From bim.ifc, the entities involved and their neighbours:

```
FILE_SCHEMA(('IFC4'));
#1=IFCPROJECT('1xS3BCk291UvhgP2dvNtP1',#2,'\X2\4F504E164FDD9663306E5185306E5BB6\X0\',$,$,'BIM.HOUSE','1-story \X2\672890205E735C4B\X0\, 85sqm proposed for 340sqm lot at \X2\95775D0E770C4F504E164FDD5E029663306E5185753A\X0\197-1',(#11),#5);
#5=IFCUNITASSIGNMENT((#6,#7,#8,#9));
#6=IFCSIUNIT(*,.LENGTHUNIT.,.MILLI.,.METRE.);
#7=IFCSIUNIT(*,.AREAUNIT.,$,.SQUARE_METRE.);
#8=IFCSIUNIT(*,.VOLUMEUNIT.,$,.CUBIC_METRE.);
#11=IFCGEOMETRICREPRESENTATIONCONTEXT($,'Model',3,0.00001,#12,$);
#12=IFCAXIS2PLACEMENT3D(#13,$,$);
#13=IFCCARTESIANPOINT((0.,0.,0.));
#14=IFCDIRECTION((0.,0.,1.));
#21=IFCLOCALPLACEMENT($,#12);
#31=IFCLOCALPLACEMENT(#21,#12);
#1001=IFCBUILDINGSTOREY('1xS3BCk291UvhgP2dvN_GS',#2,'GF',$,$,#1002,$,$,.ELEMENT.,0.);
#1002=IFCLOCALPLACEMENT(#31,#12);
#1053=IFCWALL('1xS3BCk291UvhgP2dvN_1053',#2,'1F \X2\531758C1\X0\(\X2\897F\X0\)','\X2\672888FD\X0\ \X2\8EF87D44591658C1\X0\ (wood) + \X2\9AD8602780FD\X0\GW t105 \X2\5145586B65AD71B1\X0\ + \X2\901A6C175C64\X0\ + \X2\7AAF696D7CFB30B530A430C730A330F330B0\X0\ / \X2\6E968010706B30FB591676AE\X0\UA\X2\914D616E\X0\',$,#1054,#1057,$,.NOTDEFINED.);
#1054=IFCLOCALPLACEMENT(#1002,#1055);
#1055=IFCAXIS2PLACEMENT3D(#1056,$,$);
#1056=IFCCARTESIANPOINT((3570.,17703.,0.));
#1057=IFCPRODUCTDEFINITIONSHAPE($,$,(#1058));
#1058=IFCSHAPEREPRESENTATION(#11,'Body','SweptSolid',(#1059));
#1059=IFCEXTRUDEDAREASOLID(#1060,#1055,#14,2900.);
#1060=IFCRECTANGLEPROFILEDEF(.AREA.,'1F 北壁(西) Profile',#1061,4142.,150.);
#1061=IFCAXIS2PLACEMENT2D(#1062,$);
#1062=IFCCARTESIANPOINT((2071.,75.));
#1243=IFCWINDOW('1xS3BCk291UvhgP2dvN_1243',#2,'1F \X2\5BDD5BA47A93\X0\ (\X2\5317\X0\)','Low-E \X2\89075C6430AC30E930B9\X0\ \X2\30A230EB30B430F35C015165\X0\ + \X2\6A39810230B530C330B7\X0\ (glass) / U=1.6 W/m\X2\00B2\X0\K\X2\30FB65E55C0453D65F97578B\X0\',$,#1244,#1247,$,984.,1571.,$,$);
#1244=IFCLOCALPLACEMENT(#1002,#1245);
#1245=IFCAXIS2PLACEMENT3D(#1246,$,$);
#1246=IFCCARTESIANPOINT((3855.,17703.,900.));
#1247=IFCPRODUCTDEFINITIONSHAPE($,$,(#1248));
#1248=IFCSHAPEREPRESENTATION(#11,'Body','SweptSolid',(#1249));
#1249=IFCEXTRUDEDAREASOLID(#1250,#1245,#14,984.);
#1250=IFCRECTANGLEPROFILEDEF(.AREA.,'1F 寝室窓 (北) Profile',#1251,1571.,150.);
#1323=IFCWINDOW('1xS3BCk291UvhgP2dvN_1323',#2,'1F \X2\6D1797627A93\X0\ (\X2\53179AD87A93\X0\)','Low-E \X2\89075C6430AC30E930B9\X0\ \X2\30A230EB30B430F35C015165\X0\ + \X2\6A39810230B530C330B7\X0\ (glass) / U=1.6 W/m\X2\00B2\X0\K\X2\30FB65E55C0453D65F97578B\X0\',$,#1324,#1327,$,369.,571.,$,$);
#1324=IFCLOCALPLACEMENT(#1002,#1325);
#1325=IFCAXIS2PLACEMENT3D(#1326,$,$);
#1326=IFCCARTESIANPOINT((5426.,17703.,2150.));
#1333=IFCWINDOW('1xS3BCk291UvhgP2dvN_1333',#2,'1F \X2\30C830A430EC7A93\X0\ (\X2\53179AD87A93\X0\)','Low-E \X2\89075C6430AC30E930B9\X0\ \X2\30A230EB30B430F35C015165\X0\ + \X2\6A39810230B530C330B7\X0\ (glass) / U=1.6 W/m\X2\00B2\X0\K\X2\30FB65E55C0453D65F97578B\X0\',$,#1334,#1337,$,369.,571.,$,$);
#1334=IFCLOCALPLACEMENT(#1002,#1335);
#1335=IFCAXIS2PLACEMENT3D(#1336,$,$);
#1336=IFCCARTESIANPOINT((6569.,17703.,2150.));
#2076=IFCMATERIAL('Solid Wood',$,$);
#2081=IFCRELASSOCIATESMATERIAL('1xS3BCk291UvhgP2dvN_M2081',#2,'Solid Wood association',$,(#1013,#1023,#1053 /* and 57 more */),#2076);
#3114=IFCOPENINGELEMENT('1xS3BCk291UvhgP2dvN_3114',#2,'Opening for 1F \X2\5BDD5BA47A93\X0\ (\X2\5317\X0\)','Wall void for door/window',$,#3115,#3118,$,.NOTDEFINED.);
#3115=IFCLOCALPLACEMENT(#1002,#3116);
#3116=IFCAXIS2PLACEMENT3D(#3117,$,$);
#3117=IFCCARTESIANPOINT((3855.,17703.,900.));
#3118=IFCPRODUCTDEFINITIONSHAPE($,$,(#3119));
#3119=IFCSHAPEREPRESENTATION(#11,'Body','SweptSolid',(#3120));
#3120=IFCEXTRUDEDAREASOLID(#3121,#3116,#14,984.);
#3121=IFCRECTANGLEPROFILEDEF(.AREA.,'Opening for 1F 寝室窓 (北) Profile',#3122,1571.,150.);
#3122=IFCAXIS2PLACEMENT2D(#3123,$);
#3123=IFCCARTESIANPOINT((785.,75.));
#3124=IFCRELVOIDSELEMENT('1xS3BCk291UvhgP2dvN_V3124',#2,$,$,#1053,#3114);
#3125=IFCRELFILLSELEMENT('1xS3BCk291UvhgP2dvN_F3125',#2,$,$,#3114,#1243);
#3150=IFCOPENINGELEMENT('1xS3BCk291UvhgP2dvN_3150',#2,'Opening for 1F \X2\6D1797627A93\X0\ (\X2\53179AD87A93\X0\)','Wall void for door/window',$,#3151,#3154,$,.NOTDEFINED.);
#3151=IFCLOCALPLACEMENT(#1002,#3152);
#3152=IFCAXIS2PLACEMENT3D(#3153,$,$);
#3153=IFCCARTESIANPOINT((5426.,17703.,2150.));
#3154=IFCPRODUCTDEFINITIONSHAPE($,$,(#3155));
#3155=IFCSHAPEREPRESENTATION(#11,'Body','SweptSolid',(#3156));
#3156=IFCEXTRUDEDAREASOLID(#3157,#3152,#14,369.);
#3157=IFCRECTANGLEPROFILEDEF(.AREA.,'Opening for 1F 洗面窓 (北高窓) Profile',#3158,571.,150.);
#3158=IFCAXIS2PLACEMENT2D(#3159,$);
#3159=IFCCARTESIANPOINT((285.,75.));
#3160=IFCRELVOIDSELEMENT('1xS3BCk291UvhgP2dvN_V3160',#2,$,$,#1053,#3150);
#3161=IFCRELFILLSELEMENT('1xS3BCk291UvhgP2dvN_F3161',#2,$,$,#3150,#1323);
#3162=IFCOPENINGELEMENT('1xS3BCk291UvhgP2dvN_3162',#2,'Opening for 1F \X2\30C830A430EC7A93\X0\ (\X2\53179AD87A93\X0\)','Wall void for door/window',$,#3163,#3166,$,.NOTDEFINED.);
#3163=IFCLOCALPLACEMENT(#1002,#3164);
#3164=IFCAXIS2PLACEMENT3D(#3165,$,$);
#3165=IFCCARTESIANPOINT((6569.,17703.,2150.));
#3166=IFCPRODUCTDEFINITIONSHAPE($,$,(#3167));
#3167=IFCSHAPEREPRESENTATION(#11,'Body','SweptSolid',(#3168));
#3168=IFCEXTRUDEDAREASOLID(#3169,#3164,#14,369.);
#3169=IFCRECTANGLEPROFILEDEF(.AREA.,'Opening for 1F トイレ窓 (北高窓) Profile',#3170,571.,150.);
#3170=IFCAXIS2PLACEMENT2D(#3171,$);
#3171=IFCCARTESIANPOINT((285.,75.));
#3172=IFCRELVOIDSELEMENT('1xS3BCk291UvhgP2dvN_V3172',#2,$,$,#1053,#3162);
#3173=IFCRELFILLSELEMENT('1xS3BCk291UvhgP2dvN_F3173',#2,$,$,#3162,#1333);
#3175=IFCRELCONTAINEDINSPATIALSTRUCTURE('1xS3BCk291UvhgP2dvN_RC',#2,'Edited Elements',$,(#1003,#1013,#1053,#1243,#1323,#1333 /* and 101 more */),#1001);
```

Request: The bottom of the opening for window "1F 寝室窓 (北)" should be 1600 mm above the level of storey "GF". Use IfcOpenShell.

```python
import numpy as np
import ifcopenshell
import ifcopenshell.api.geometry
import ifcopenshell.geom
import ifcopenshell.util.element
import ifcopenshell.util.placement
import ifcopenshell.util.shape
import ifcopenshell.util.unit

model = ifcopenshell.open("bim.ifc")
unit_scale = ifcopenshell.util.unit.calculate_unit_scale(model)

window = model.by_id(1243)
opening = window.FillsVoids[0].RelatingOpeningElement
storey = ifcopenshell.util.element.get_container(window, ifc_class="IfcBuildingStorey")
level = ifcopenshell.util.placement.get_local_placement(storey.ObjectPlacement)[2, 3]

# The opening's origin need not be at the sill, so measure its lowest point.
shape = ifcopenshell.geom.create_shape(ifcopenshell.geom.settings(), opening)
bottom = ifcopenshell.util.shape.get_shape_bottom_elevation(shape, shape.geometry) / unit_scale
dz = level + 1.6 / unit_scale - bottom

shift = np.array([0.0, 0.0, dz])
# The window is not placed relative to its opening, so move both.
for product in (opening, window):
    matrix = ifcopenshell.util.placement.get_local_placement(product.ObjectPlacement)
    matrix[:3, 3] += shift
    ifcopenshell.api.geometry.edit_object_placement(model, product=product, matrix=matrix, is_si=False)

print(f"moved by {dz * unit_scale:+.3f} m")

model.write("bim_v2.ifc")
```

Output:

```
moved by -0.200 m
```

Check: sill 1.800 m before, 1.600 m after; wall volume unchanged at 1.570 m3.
